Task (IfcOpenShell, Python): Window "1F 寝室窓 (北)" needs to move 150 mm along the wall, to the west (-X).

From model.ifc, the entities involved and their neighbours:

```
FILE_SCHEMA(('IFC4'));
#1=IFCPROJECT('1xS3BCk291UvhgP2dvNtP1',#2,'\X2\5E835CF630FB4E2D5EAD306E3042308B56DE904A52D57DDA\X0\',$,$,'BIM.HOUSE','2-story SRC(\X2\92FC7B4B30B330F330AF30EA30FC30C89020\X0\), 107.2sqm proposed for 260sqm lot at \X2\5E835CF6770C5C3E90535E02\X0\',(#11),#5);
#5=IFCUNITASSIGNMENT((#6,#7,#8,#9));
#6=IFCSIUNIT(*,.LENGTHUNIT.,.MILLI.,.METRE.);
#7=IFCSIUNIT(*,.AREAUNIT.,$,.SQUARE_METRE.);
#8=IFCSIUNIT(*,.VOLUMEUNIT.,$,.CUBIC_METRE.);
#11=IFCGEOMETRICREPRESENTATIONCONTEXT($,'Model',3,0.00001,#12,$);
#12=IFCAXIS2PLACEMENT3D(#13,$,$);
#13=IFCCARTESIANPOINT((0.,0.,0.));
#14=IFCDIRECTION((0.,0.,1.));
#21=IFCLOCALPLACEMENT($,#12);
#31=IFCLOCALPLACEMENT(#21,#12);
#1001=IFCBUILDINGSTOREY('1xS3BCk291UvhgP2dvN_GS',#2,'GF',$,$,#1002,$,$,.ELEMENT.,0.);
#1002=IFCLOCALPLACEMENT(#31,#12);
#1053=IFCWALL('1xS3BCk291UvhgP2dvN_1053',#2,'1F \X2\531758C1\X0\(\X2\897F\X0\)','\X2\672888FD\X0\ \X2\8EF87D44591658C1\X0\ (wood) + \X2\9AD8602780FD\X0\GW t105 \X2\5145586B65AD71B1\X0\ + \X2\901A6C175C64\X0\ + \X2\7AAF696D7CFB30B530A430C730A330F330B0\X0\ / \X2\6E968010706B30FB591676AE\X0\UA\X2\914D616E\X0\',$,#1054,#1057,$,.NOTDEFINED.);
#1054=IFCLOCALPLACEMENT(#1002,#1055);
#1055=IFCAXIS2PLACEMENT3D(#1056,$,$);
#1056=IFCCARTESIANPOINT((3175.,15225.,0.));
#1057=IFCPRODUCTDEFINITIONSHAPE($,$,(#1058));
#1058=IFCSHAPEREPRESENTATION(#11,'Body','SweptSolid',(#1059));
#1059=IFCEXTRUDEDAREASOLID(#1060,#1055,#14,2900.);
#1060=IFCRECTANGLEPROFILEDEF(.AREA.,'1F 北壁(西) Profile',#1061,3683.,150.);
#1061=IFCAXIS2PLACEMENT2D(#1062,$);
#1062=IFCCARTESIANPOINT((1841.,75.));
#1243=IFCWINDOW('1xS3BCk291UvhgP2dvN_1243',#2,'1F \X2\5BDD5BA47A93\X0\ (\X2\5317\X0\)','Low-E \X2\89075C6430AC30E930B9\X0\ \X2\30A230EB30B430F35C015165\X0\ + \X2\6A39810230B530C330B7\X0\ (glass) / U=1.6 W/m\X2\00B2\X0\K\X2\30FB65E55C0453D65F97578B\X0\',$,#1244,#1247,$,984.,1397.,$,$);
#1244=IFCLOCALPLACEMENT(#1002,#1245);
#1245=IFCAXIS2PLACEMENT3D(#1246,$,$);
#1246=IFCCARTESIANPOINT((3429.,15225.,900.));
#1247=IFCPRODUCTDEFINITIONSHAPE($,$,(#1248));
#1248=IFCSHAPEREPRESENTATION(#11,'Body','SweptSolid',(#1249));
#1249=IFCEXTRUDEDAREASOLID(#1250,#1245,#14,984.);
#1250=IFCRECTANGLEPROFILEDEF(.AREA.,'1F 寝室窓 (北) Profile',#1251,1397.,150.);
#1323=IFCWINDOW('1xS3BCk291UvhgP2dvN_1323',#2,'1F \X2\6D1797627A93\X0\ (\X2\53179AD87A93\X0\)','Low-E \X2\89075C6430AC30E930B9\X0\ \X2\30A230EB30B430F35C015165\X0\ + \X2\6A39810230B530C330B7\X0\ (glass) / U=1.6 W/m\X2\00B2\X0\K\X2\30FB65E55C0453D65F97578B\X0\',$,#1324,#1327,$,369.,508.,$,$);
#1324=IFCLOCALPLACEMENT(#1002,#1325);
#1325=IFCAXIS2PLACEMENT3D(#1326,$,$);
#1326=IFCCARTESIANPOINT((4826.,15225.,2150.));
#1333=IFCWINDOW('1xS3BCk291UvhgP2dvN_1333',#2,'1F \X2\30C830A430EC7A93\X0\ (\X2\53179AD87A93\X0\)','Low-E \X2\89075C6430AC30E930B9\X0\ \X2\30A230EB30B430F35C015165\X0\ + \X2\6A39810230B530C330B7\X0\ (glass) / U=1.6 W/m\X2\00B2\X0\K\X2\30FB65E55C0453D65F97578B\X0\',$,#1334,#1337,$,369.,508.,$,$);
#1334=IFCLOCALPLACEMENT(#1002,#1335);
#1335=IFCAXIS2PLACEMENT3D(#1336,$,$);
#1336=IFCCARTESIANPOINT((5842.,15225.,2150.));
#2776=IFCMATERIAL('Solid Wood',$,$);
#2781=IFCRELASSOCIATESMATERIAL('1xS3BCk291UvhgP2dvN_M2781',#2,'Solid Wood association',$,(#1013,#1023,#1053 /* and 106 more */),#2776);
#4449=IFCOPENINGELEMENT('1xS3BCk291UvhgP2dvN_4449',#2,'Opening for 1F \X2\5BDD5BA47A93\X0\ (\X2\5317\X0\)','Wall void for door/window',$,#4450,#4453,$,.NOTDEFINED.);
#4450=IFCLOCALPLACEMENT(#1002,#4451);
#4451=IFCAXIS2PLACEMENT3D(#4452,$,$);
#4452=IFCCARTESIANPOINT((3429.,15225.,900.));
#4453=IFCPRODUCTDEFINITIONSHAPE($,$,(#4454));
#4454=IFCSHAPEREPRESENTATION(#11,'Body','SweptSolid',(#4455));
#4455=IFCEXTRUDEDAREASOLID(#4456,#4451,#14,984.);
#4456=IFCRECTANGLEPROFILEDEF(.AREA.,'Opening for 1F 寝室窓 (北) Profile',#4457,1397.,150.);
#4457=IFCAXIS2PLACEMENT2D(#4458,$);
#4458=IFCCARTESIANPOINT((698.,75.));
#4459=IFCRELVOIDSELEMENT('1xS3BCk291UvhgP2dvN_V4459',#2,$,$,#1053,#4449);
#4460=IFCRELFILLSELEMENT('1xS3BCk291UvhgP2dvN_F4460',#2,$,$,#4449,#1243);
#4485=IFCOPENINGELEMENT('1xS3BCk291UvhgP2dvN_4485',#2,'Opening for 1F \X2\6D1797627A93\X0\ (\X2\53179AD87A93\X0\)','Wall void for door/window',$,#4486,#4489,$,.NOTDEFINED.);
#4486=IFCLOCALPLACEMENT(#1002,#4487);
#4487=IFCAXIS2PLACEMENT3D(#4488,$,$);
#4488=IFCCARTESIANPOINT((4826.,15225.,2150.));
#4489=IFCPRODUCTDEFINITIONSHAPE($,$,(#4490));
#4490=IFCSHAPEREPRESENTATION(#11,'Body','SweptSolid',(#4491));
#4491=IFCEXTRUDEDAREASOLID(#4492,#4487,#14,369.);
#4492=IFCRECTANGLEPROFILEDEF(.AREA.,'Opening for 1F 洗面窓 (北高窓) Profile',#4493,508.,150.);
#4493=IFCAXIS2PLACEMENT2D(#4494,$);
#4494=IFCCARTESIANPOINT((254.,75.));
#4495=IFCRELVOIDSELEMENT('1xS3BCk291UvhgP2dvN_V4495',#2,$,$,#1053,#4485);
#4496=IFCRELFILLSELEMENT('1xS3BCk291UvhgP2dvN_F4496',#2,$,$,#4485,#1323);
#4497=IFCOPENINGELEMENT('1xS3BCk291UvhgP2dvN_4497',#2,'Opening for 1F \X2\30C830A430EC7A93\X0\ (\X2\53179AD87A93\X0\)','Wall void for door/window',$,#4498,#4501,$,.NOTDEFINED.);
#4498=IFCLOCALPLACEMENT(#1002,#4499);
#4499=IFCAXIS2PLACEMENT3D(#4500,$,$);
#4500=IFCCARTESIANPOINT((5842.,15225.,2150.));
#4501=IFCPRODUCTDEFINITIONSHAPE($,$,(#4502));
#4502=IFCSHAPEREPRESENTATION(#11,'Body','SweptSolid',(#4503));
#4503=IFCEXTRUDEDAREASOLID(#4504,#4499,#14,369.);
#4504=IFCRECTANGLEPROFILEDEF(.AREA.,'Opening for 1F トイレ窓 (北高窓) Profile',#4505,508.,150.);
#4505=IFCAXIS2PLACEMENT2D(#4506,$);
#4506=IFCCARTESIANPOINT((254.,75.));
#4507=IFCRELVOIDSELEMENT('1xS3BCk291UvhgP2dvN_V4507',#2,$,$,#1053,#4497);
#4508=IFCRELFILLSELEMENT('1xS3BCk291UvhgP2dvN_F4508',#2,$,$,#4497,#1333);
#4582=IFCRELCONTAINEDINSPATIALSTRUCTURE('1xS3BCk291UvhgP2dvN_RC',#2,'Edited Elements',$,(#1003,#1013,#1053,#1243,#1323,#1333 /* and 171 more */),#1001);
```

```python
import ifcopenshell
import ifcopenshell.api.geometry
import ifcopenshell.util.placement
import ifcopenshell.util.unit

model = ifcopenshell.open("model.ifc")
unit_scale = ifcopenshell.util.unit.calculate_unit_scale(model)

window = model.by_guid("1xS3BCk291UvhgP2dvN_1243")
opening = window.FillsVoids[0].RelatingOpeningElement
wall = opening.VoidsElements[0].RelatingBuildingElement

wall_matrix = ifcopenshell.util.placement.get_local_placement(wall.ObjectPlacement)
shift = wall_matrix[:3, 0] * -0.15 / unit_scale
before = ifcopenshell.util.placement.get_local_placement(window.ObjectPlacement)[:3, 3].copy()

# The window is not placed relative to its opening, so move both.
for product in (opening, window):
    matrix = ifcopenshell.util.placement.get_local_placement(product.ObjectPlacement)
    matrix[:3, 3] += shift
    ifcopenshell.api.geometry.edit_object_placement(model, product=product, matrix=matrix, is_si=False)

after = ifcopenshell.util.placement.get_local_placement(window.ObjectPlacement)[:3, 3]
print("window moved by", (after - before).round(3) + 0.0)

model.write("model-out.ifc")
```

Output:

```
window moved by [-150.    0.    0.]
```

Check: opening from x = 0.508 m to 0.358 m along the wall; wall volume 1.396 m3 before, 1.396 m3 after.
